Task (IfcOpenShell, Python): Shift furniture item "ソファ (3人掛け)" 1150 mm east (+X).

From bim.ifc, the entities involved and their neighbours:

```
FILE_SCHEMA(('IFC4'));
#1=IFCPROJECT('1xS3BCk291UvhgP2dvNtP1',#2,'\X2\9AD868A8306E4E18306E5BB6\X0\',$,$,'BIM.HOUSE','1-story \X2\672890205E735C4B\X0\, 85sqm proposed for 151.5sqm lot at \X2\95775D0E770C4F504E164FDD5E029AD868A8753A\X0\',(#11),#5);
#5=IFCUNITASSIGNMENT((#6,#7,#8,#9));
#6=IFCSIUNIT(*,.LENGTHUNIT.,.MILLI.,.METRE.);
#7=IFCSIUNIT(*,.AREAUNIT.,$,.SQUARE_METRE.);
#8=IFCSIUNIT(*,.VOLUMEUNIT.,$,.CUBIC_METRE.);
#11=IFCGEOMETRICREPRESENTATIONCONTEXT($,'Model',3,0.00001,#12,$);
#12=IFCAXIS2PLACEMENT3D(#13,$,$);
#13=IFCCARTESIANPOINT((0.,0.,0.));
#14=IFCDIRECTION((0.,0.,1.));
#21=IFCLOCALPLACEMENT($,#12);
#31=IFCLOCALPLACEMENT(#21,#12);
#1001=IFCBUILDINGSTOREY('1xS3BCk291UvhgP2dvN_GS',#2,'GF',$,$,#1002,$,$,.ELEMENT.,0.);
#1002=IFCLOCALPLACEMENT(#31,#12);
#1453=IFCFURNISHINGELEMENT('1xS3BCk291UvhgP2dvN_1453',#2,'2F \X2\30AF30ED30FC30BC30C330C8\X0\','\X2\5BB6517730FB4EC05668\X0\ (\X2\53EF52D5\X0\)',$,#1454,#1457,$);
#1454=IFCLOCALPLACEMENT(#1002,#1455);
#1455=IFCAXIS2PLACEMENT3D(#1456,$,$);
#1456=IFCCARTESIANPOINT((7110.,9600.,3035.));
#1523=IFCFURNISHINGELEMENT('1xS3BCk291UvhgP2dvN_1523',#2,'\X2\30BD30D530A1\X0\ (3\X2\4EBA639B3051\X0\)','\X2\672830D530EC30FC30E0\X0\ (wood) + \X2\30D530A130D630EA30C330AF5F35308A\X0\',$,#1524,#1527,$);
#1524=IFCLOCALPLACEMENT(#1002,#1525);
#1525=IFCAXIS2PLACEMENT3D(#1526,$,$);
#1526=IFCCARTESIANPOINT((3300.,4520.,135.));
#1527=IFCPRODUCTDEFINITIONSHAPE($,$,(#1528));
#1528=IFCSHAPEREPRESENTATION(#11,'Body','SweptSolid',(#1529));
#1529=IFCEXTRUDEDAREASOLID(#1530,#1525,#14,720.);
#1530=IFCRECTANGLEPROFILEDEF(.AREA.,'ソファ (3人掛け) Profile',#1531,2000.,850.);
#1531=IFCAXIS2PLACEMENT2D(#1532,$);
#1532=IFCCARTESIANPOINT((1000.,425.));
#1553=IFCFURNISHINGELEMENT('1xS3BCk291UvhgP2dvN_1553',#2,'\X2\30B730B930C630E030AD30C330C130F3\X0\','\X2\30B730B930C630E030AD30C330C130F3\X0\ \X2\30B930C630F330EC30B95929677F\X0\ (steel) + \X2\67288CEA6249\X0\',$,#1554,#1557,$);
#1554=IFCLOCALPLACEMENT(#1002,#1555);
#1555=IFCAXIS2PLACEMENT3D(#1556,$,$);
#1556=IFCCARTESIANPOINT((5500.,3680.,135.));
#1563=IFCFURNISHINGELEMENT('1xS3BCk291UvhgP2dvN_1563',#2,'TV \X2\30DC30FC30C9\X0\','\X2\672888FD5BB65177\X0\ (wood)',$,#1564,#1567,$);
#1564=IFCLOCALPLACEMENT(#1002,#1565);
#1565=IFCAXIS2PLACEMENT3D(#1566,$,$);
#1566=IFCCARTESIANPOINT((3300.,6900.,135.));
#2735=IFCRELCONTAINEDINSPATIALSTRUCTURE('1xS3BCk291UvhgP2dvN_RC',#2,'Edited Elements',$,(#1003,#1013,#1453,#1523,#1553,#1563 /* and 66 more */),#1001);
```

```python
import ifcopenshell
import ifcopenshell.api.geometry
import ifcopenshell.util.placement
import ifcopenshell.util.unit

model = ifcopenshell.open("bim.ifc")
unit_scale = ifcopenshell.util.unit.calculate_unit_scale(model)

item = model.by_id(1523)
matrix = ifcopenshell.util.placement.get_local_placement(item.ObjectPlacement)
matrix[0, 3] += 1.15 / unit_scale
ifcopenshell.api.geometry.edit_object_placement(model, product=item, matrix=matrix, is_si=False)

print(ifcopenshell.util.placement.get_local_placement(item.ObjectPlacement).round(3) + 0.0)

model.write("bim_updated.ifc")
```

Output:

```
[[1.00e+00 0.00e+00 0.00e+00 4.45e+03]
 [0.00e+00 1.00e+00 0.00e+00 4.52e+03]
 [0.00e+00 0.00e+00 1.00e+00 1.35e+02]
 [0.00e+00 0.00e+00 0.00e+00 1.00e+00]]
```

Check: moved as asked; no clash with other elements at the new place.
